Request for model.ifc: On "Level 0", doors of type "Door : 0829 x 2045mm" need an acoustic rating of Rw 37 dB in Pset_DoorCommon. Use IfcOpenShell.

First a look at what the model holds.

```python
import ifcopenshell
import ifcopenshell.util.element

model = ifcopenshell.open("model.ifc")
print(model.schema)
storey = next(s for s in model.by_type("IfcBuildingStorey") if s.Name == "Level 0")
doors = [e for e in ifcopenshell.util.element.get_decomposition(storey) if e.is_a("IfcDoor")]
seen = {}
for e in doors:
    element_type = ifcopenshell.util.element.get_type(e)
    key = (element_type.Name if element_type != e and element_type else None, ifcopenshell.util.element.get_pset(e, "Pset_DoorCommon", "AcousticRating"))
    seen[key] = seen.get(key, 0) + 1
for (name, value), count in sorted(seen.items(), key=str):
    print(count, "x", name, "|", value)
```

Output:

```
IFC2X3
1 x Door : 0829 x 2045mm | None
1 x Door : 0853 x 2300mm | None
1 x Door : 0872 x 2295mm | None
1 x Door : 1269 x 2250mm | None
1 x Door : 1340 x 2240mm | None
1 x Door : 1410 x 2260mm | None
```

```python
import ifcopenshell
import ifcopenshell.api.pset
import ifcopenshell.util.element

model = ifcopenshell.open("model.ifc")

storey = next(s for s in model.by_type("IfcBuildingStorey") if s.Name == "Level 0")
doors = [e for e in ifcopenshell.util.element.get_decomposition(storey) if e.is_a("IfcDoor")]

count = 0
for e in doors:
    element_type = ifcopenshell.util.element.get_type(e)
    if element_type in (None, e) or element_type.Name != "Door : 0829 x 2045mm":
        continue
    # add_pset returns the element's existing set when there is one.
    pset = ifcopenshell.api.pset.add_pset(model, product=e, name="Pset_DoorCommon")
    ifcopenshell.api.pset.edit_pset(model, pset=pset, properties={"AcousticRating": "Rw 37 dB"})
    count += 1

print(count, "doors updated")

model.write("model_edited.ifc")
```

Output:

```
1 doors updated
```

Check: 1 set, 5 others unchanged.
